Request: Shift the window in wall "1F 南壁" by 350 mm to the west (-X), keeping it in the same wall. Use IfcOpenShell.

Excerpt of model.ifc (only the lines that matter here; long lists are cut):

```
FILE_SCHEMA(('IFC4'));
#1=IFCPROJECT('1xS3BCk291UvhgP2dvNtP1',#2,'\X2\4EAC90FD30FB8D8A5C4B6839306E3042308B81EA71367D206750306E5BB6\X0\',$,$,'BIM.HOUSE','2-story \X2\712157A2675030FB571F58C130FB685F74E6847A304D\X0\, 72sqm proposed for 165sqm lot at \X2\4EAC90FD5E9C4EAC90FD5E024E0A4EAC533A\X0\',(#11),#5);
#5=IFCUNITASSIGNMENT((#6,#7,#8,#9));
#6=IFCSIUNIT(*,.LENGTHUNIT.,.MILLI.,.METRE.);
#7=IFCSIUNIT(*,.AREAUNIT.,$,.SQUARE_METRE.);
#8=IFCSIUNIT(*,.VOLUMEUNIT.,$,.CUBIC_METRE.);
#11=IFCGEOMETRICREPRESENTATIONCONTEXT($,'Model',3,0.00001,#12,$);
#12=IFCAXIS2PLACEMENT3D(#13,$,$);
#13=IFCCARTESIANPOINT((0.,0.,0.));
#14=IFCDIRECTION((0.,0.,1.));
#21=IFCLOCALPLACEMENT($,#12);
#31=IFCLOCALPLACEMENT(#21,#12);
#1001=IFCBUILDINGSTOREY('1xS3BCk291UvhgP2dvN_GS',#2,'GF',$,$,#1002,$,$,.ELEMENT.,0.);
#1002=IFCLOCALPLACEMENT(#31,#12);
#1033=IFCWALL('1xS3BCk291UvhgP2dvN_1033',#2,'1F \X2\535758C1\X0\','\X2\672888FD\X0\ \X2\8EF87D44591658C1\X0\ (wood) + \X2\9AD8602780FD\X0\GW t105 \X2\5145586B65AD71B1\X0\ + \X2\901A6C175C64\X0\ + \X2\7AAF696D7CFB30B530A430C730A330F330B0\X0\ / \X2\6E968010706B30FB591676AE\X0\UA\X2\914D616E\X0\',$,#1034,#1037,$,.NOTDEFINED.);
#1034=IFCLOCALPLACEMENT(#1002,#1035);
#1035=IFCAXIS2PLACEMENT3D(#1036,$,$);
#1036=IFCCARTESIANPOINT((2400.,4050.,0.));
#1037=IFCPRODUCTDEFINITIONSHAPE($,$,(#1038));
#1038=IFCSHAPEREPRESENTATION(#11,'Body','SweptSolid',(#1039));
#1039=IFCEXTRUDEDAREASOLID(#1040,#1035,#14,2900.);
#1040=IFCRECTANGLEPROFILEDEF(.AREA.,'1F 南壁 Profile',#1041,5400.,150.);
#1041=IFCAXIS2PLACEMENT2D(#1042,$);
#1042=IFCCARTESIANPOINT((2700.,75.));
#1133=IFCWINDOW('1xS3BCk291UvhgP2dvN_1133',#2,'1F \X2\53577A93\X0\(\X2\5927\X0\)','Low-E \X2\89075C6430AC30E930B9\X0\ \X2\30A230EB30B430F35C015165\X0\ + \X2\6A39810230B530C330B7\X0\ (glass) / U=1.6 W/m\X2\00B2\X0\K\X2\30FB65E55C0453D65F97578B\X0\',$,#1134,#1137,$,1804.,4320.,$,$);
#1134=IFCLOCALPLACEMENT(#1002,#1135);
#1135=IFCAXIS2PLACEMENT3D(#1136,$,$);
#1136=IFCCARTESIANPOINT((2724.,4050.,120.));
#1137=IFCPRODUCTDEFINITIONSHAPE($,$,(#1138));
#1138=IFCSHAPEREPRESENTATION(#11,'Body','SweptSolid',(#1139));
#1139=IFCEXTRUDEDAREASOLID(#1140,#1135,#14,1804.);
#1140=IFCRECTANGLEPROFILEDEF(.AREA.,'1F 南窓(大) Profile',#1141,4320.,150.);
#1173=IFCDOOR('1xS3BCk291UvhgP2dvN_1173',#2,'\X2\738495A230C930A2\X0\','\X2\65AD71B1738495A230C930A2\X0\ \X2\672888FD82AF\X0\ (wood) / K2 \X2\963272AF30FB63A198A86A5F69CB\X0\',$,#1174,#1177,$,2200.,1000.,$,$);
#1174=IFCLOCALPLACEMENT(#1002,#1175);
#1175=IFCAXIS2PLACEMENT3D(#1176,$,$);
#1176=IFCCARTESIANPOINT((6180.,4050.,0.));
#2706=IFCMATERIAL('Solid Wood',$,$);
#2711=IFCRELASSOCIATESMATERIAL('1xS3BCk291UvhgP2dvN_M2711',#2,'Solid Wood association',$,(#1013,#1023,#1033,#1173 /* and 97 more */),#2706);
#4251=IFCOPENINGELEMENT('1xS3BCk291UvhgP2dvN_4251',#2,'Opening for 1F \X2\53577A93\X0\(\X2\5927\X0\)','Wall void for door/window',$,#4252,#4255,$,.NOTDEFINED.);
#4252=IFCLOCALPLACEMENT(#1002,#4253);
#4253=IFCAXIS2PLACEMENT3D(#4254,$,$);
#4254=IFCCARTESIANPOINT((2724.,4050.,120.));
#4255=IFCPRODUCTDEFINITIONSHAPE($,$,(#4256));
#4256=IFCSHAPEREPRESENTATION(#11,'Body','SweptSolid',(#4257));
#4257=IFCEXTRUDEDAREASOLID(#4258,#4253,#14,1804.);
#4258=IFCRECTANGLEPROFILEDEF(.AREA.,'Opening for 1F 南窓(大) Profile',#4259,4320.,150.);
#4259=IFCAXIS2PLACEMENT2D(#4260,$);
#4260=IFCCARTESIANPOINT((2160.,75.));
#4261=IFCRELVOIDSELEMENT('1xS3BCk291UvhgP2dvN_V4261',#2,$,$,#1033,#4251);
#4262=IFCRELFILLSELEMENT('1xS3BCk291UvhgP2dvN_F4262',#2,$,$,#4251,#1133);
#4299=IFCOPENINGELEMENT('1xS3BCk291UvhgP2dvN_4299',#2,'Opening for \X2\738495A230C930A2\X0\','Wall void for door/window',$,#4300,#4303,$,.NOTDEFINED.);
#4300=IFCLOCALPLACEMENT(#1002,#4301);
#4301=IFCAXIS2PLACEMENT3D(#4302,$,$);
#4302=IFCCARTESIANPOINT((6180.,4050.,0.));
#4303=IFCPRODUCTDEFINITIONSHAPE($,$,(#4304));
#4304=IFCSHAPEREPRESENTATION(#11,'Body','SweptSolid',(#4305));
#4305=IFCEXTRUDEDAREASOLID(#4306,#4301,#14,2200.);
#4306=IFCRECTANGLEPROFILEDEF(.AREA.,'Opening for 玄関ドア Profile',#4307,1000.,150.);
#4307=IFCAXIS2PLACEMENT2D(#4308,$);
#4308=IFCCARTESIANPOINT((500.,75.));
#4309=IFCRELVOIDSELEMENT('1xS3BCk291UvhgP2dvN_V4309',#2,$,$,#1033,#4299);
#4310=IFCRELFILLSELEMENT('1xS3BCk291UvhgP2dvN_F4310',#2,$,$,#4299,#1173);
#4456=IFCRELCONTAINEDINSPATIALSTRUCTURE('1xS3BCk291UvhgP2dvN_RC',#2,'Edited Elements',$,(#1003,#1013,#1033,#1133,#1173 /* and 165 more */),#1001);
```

```python
import ifcopenshell
import ifcopenshell.api.geometry
import ifcopenshell.util.placement
import ifcopenshell.util.unit

model = ifcopenshell.open("model.ifc")
unit_scale = ifcopenshell.util.unit.calculate_unit_scale(model)

window = model.by_guid("1xS3BCk291UvhgP2dvN_1133")
opening = window.FillsVoids[0].RelatingOpeningElement
wall = opening.VoidsElements[0].RelatingBuildingElement

wall_matrix = ifcopenshell.util.placement.get_local_placement(wall.ObjectPlacement)
shift = wall_matrix[:3, 0] * -0.35 / unit_scale
before = ifcopenshell.util.placement.get_local_placement(window.ObjectPlacement)[:3, 3].copy()

# The window is not placed relative to its opening, so move both.
for product in (opening, window):
    matrix = ifcopenshell.util.placement.get_local_placement(product.ObjectPlacement)
    matrix[:3, 3] += shift
    ifcopenshell.api.geometry.edit_object_placement(model, product=product, matrix=matrix, is_si=False)

after = ifcopenshell.util.placement.get_local_placement(window.ObjectPlacement)[:3, 3]
print("window moved by", (after - before).round(3) + 0.0)

model.write("model_updated.ifc")
```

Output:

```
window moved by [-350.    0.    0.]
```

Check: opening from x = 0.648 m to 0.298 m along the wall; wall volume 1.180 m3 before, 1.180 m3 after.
